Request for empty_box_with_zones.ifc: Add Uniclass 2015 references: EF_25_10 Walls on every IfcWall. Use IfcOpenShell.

First a look at what the model holds.

```python
import ifcopenshell

model = ifcopenshell.open("empty_box_with_zones.ifc")
print(model.schema)
print("classifications:", [c.Name for c in model.by_type("IfcClassification")])
for ifc_class in ("IfcDoor", "IfcRoof", "IfcStair", "IfcWall", "IfcWindow"):
    print(ifc_class, len(model.by_type(ifc_class)))
```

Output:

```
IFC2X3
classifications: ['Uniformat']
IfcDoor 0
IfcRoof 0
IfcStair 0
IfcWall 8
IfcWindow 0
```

```python
import ifcopenshell
import ifcopenshell.api.classification

model = ifcopenshell.open("empty_box_with_zones.ifc")

# IFC2X3 requires Source and Edition and has no link from the project to the system.
system = model.create_entity("IfcClassification", Source="NBS", Edition="2015", Name="Uniclass 2015")

codes = {
    "IfcWall": ("EF_25_10", "Walls"),
}
for ifc_class, (code, name) in codes.items():
    products = model.by_type(ifc_class)
    ifcopenshell.api.classification.add_reference(
        model, products=products, classification=system, identification=code, name=name
    )
    print(code, len(products))

model.write("empty_box_with_zones_updated.ifc")
```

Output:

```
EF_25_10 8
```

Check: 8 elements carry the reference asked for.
